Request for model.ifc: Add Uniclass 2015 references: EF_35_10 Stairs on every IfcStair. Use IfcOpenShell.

First a look at what the model holds.

```python
import ifcopenshell

model = ifcopenshell.open("model.ifc")
print(model.schema)
print("classifications:", [c.Name for c in model.by_type("IfcClassification")])
for ifc_class in ("IfcDoor", "IfcRoof", "IfcStair", "IfcWall", "IfcWindow"):
    print(ifc_class, len(model.by_type(ifc_class)))
```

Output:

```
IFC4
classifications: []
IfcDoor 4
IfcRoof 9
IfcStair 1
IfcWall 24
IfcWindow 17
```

```python
import ifcopenshell
import ifcopenshell.api.classification

model = ifcopenshell.open("model.ifc")

system = ifcopenshell.api.classification.add_classification(model, classification="Uniclass 2015")

codes = {
    "IfcStair": ("EF_35_10", "Stairs"),
}
for ifc_class, (code, name) in codes.items():
    products = model.by_type(ifc_class)
    ifcopenshell.api.classification.add_reference(
        model, products=products, classification=system, identification=code, name=name
    )
    print(code, len(products))

model.write("model-out.ifc")
```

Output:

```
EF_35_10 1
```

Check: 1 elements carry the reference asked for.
